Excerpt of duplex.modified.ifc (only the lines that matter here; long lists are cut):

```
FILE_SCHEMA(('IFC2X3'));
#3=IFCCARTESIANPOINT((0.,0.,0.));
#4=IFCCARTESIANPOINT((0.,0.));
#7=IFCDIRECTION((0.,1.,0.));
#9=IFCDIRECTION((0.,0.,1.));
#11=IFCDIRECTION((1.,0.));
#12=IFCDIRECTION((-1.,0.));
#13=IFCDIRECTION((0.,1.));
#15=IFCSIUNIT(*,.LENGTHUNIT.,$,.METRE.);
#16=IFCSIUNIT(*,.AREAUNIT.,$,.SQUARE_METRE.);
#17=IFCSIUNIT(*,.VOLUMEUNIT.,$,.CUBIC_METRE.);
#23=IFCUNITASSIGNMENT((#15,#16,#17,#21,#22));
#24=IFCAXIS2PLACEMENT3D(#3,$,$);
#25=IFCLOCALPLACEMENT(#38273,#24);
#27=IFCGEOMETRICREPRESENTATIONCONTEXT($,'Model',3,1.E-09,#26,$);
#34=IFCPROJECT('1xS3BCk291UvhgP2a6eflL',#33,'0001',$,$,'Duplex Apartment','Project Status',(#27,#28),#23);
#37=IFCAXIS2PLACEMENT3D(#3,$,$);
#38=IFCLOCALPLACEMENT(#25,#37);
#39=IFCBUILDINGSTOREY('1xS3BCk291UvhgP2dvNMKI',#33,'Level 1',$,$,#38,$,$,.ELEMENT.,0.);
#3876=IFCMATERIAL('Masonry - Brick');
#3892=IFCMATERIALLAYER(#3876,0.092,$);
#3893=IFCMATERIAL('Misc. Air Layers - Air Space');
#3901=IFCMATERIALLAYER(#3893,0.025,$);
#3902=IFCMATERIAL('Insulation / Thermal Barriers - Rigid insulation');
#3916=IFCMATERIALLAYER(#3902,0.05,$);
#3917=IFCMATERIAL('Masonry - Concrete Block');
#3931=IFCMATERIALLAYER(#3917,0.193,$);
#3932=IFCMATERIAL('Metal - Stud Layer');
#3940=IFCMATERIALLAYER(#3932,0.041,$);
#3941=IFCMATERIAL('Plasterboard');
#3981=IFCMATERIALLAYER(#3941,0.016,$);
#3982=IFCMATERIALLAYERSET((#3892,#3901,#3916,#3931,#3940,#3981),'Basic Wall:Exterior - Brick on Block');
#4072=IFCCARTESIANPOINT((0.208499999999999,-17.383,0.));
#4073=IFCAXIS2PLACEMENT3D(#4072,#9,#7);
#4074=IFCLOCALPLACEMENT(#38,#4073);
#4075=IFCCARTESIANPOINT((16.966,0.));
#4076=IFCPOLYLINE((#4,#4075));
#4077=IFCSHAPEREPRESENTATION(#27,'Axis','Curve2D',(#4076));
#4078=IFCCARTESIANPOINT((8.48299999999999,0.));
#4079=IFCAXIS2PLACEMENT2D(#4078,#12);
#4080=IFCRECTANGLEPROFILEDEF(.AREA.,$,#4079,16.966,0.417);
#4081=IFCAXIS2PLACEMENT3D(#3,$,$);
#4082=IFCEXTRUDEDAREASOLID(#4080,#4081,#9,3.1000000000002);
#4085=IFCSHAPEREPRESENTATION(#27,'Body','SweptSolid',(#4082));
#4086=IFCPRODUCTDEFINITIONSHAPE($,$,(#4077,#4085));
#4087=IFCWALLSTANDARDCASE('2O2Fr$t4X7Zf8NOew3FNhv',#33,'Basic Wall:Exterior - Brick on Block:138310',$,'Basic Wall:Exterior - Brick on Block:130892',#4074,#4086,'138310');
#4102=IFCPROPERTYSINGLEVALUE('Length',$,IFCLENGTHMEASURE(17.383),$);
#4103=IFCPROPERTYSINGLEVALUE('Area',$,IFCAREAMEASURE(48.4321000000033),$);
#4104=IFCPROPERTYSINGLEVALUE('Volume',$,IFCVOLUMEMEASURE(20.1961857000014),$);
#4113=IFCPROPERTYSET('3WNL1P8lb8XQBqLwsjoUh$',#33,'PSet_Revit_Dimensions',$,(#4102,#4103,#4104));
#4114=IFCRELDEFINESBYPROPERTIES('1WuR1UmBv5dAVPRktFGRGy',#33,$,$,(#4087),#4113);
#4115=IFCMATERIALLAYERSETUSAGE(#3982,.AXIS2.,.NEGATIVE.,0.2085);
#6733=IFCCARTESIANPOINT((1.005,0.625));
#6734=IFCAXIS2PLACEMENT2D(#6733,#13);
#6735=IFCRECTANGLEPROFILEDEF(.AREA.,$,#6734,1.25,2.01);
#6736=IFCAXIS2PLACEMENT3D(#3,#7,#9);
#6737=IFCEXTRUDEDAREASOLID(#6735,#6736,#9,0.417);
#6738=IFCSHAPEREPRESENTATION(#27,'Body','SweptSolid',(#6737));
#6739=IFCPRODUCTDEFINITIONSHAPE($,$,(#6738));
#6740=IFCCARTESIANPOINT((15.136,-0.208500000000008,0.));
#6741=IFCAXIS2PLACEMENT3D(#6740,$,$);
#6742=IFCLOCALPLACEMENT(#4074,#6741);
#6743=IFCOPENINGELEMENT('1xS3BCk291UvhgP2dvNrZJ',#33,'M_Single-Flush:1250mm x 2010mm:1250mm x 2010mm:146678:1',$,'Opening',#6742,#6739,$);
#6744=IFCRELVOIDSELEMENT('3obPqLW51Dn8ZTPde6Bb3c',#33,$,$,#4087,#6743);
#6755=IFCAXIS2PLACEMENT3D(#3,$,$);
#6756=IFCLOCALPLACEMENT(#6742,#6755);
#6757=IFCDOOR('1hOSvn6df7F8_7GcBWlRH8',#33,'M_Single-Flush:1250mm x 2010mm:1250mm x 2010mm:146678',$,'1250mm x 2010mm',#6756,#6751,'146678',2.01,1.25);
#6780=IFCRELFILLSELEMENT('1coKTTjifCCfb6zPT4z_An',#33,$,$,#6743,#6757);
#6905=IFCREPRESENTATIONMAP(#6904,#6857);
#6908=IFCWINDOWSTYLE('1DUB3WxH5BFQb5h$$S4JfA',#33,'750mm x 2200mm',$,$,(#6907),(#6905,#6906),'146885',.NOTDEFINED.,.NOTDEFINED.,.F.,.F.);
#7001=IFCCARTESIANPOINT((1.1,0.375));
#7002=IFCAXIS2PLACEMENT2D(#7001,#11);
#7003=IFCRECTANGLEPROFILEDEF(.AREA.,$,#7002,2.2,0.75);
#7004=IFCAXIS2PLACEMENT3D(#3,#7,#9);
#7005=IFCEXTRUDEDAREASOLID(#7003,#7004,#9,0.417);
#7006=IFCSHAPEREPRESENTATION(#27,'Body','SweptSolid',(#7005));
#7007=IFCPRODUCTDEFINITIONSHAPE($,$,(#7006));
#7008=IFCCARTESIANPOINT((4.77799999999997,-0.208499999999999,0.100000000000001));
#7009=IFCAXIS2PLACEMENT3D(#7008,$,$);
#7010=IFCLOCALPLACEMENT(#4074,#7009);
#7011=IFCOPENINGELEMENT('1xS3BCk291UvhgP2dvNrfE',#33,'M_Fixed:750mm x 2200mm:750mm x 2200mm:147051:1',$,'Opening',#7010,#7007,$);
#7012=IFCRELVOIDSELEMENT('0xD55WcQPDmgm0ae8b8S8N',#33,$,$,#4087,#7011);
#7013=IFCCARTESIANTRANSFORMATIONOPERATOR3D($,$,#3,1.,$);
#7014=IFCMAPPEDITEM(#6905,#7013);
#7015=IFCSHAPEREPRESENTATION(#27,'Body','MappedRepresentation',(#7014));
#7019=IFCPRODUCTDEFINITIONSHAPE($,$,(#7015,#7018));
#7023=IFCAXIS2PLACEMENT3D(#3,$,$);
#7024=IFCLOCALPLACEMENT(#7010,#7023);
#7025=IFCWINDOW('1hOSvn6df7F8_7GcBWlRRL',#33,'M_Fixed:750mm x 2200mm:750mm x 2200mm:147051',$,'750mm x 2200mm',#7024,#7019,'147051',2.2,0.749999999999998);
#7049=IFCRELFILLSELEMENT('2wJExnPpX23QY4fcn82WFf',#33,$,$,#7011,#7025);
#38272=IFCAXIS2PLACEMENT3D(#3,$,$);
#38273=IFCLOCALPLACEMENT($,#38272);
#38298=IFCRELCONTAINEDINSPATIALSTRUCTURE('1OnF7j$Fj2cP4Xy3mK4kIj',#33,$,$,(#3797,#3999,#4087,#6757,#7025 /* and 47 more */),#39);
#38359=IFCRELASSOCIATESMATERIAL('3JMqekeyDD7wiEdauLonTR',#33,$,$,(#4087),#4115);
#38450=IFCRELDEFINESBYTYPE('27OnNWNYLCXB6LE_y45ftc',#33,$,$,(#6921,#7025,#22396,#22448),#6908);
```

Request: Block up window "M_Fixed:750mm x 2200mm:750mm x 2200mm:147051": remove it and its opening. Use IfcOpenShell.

```python
import ifcopenshell
import ifcopenshell.api.feature
import ifcopenshell.api.pset
import ifcopenshell.api.root
import ifcopenshell.geom
import ifcopenshell.util.element
import ifcopenshell.util.shape
import ifcopenshell.util.unit

model = ifcopenshell.open("duplex.modified.ifc")
area_scale = ifcopenshell.util.unit.calculate_unit_scale(model, "AREAUNIT")
volume_scale = ifcopenshell.util.unit.calculate_unit_scale(model, "VOLUMEUNIT")
settings = ifcopenshell.geom.settings()


def volume(element):
    """Net volume in cubic metres, openings subtracted."""
    shape = ifcopenshell.geom.create_shape(settings, element)
    return ifcopenshell.util.shape.get_volume(shape.geometry)


window = model.by_guid("1hOSvn6df7F8_7GcBWlRRL")
opening = window.FillsVoids[0].RelatingOpeningElement
wall = opening.VoidsElements[0].RelatingBuildingElement
before = volume(wall)

ifcopenshell.api.root.remove_product(model, product=window)
ifcopenshell.api.feature.remove_feature(model, feature=opening)

after = volume(wall)
thickness = 0.417  # wall thickness in metres

# Update the wall's stored quantities.
pset = model.by_id(ifcopenshell.util.element.get_pset(wall, "PSet_Revit_Dimensions", should_inherit=False)["id"])
ifcopenshell.api.pset.edit_pset(model, pset=pset, properties={
    "Area": model.create_entity("IfcAreaMeasure", after / thickness / area_scale),
    "Volume": model.create_entity("IfcVolumeMeasure", after / volume_scale),
})

print(f"wall volume {before:.3f} -> {after:.3f} m3")

model.write("duplex.modified_rev.ifc")
```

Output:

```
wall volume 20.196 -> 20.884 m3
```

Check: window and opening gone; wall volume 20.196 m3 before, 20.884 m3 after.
